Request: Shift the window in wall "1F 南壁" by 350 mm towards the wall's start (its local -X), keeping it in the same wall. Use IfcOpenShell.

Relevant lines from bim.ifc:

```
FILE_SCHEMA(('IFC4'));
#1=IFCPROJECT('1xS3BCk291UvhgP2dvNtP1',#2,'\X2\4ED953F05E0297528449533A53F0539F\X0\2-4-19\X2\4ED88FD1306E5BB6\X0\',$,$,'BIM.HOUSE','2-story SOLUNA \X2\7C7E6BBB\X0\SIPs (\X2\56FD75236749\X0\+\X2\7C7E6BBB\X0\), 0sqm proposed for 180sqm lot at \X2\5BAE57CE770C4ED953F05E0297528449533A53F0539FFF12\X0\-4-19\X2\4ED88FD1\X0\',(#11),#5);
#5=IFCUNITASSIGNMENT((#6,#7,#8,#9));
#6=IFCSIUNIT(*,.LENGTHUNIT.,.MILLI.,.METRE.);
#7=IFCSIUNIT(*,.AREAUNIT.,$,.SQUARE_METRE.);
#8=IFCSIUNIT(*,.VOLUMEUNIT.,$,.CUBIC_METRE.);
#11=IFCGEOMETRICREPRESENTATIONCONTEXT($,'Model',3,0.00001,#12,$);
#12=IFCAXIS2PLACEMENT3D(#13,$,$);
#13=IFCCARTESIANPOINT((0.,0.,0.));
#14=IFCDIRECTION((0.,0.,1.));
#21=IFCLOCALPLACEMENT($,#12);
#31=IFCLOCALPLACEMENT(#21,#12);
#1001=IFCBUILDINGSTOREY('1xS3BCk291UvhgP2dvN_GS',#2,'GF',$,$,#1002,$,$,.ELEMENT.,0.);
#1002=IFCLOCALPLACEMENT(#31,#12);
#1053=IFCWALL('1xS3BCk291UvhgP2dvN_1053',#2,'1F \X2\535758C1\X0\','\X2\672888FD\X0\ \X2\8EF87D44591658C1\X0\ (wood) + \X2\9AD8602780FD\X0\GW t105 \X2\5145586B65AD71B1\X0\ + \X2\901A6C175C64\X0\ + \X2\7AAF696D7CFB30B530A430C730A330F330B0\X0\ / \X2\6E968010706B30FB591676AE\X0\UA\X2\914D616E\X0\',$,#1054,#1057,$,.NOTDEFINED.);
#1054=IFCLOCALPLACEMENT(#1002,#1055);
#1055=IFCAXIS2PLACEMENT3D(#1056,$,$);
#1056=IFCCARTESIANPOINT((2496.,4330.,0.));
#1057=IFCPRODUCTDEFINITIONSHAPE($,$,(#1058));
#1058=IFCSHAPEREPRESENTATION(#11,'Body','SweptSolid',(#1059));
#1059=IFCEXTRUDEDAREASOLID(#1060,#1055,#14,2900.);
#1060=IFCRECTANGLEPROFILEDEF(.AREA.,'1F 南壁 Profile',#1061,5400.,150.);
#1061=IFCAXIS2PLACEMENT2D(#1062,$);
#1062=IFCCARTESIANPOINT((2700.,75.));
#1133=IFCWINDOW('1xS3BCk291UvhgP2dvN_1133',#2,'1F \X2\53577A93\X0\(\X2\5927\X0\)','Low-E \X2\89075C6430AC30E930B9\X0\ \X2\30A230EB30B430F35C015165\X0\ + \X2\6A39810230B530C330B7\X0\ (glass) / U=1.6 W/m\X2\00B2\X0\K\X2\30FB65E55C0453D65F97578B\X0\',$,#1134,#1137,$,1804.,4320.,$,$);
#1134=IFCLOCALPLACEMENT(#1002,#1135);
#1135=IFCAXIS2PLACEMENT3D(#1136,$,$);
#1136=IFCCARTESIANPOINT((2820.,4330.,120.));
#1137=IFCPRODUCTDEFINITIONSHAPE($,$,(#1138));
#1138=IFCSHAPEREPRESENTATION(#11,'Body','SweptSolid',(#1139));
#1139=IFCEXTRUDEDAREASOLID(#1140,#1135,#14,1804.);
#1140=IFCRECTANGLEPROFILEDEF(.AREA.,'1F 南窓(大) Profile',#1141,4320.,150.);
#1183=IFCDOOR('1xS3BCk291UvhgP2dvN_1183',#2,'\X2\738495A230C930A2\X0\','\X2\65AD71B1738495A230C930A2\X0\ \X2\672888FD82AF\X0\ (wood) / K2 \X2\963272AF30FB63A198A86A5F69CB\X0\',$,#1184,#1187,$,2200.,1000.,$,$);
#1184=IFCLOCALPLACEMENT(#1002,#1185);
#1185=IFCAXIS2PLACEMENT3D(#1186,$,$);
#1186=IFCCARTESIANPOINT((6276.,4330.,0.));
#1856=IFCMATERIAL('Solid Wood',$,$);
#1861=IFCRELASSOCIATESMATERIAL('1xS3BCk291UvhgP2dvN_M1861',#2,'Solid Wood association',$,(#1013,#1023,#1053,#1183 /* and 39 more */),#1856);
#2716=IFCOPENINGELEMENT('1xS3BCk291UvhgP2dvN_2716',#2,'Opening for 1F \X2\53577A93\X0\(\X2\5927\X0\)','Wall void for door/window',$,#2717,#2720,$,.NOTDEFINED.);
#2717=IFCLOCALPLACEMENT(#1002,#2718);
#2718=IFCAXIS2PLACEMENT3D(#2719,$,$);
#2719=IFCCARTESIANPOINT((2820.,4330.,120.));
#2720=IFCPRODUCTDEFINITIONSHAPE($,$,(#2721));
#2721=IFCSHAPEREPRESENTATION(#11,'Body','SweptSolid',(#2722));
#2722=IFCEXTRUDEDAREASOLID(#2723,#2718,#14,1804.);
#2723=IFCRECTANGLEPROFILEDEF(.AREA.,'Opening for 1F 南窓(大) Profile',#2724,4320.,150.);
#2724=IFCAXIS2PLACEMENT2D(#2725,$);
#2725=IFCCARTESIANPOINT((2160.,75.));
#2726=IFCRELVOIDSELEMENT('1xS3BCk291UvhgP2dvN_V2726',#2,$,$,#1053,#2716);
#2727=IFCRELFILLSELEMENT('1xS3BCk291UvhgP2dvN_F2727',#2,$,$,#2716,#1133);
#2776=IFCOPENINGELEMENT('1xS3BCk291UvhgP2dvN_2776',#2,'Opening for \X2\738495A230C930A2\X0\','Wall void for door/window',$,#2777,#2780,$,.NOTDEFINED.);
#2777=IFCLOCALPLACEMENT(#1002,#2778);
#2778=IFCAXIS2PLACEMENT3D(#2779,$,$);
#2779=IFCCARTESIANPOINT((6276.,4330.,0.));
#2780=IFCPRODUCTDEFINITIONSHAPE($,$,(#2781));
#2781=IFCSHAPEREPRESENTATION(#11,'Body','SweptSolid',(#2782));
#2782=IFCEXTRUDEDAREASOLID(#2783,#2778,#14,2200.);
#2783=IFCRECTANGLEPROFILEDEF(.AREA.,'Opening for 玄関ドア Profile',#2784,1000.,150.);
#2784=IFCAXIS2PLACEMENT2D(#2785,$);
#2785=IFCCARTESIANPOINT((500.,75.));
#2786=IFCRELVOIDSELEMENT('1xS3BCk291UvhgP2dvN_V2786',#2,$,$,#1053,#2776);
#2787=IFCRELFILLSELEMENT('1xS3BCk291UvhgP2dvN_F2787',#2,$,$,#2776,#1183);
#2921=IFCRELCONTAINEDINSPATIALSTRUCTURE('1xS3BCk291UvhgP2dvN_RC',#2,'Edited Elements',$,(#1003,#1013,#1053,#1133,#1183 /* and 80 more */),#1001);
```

```python
import ifcopenshell
import ifcopenshell.api.geometry
import ifcopenshell.util.placement
import ifcopenshell.util.unit

model = ifcopenshell.open("bim.ifc")
unit_scale = ifcopenshell.util.unit.calculate_unit_scale(model)

window = model.by_id(1133)
opening = window.FillsVoids[0].RelatingOpeningElement
wall = opening.VoidsElements[0].RelatingBuildingElement

wall_matrix = ifcopenshell.util.placement.get_local_placement(wall.ObjectPlacement)
shift = wall_matrix[:3, 0] * -0.35 / unit_scale
before = ifcopenshell.util.placement.get_local_placement(window.ObjectPlacement)[:3, 3].copy()

# The window is not placed relative to its opening, so move both.
for product in (opening, window):
    matrix = ifcopenshell.util.placement.get_local_placement(product.ObjectPlacement)
    matrix[:3, 3] += shift
    ifcopenshell.api.geometry.edit_object_placement(model, product=product, matrix=matrix, is_si=False)

after = ifcopenshell.util.placement.get_local_placement(window.ObjectPlacement)[:3, 3]
print("window moved by", (after - before).round(3) + 0.0)

model.write("bim_updated.ifc")
```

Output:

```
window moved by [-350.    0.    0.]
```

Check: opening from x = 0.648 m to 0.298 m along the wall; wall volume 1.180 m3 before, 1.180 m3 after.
